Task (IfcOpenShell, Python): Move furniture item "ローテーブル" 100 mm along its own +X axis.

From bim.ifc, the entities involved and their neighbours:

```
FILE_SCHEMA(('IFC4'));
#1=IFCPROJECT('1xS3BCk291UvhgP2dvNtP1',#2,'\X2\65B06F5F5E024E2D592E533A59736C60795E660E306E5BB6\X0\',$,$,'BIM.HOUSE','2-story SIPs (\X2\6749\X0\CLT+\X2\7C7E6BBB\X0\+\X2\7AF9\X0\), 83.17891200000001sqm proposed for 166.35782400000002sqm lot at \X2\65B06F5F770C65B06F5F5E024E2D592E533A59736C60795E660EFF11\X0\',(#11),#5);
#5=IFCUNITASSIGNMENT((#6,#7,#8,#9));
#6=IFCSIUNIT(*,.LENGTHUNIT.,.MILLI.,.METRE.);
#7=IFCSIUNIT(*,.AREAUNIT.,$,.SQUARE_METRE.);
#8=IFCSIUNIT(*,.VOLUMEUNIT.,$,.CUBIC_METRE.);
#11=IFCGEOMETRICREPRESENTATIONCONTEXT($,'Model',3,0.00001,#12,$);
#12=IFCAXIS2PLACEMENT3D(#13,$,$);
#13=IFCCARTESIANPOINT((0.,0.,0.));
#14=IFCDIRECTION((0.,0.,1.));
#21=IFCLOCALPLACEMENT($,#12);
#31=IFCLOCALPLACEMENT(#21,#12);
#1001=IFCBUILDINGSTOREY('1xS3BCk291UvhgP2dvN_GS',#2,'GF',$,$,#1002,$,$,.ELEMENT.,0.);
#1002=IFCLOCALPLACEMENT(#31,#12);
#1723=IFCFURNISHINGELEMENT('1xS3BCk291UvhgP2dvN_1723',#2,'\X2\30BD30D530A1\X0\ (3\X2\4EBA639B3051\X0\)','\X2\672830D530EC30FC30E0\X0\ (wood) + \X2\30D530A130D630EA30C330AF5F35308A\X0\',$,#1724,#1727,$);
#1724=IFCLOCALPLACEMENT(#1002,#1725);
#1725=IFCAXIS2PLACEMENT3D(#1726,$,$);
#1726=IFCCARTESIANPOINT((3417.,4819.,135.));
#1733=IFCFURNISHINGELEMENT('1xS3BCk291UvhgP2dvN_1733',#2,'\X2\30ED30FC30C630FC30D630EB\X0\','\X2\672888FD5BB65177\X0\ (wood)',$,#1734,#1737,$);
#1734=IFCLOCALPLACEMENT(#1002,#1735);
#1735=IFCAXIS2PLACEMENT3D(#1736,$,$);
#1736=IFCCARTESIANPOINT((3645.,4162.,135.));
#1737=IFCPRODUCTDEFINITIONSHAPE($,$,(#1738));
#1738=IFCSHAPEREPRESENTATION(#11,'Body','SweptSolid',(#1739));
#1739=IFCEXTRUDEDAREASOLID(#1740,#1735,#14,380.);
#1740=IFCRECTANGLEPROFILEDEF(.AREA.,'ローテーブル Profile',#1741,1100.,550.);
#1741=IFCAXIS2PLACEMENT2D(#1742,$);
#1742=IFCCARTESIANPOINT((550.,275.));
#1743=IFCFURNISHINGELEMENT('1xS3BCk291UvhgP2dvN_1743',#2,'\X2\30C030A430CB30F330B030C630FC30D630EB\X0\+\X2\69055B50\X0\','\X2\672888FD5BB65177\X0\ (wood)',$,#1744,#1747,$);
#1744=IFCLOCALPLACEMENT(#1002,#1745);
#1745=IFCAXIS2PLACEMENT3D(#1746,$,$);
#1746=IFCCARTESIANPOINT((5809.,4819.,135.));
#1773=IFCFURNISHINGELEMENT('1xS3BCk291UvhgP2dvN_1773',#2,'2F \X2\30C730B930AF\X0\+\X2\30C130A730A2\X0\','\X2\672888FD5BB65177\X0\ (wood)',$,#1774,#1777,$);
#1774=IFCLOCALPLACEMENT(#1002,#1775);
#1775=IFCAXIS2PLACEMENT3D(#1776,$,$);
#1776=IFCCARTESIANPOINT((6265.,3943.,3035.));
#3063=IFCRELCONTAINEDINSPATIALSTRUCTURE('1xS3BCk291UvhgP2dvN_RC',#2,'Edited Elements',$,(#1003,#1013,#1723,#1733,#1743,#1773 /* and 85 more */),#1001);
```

```python
import ifcopenshell
import ifcopenshell.api.geometry
import ifcopenshell.util.placement

model = ifcopenshell.open("bim.ifc")

item = model.by_guid("1xS3BCk291UvhgP2dvN_1733")
matrix = ifcopenshell.util.placement.get_local_placement(item.ObjectPlacement)
matrix[:3, 3] += matrix[:3, 0] * 100.0
ifcopenshell.api.geometry.edit_object_placement(model, product=item, matrix=matrix, is_si=False)

print(ifcopenshell.util.placement.get_local_placement(item.ObjectPlacement).round(3) + 0.0)

model.write("bim_updated.ifc")
```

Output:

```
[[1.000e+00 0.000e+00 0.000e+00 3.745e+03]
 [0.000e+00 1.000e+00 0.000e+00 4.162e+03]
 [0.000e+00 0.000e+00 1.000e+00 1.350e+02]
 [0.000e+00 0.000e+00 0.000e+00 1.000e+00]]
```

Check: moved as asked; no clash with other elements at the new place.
